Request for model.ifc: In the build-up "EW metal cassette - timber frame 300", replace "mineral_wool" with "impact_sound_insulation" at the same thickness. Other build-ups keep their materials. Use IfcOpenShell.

First a look at what the model holds.

```python
import ifcopenshell
import ifcopenshell.util.element

model = ifcopenshell.open("model.ifc")
print(model.schema)
for layer_set in model.by_type("IfcMaterialLayerSet"):
    if layer_set.LayerSetName == "EW metal cassette - timber frame 300":
        for layer in layer_set.MaterialLayers:
            print(layer.id(), layer.Material and layer.Material.Name, layer.LayerThickness, sep=" | ")
        print(len(ifcopenshell.util.element.get_elements_by_material(model, layer_set)), "elements and types use it")
print(sorted(m.Name for m in model.by_type("IfcMaterial") if m.Name)[:60])
```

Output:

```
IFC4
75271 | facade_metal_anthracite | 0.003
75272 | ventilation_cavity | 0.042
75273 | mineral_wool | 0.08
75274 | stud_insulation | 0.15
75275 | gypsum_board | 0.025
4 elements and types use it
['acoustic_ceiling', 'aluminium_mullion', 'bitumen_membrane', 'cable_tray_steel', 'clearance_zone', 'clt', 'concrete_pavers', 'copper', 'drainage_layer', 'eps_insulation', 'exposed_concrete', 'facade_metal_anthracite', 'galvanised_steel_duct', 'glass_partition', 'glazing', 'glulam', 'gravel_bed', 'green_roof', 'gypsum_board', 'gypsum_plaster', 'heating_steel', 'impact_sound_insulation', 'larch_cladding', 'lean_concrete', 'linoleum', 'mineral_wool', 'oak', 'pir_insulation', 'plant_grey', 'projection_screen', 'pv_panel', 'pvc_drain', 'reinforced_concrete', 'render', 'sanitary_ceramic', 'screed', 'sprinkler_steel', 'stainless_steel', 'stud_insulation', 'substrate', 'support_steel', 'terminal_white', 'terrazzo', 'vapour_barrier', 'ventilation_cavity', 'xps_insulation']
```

```python
import ifcopenshell
import ifcopenshell.api.material

model = ifcopenshell.open("model.ifc")

layer_set = next(s for s in model.by_type("IfcMaterialLayerSet") if s.LayerSetName == "EW metal cassette - timber frame 300")
layer = next(l for l in layer_set.MaterialLayers if l.Material and l.Material.Name == "mineral_wool")
material = next(m for m in model.by_type("IfcMaterial") if m.Name == "impact_sound_insulation")

# Point this one layer at the other material; renaming the old one would change it everywhere.
ifcopenshell.api.material.edit_layer(model, layer=layer, attributes={"Name": material.Name}, material=material)

print([l.Material.Name if l.Material else None for l in layer_set.MaterialLayers])

model.write("model-out.ifc")
```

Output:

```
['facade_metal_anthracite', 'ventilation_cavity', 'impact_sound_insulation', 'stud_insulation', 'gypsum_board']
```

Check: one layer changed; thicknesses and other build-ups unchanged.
